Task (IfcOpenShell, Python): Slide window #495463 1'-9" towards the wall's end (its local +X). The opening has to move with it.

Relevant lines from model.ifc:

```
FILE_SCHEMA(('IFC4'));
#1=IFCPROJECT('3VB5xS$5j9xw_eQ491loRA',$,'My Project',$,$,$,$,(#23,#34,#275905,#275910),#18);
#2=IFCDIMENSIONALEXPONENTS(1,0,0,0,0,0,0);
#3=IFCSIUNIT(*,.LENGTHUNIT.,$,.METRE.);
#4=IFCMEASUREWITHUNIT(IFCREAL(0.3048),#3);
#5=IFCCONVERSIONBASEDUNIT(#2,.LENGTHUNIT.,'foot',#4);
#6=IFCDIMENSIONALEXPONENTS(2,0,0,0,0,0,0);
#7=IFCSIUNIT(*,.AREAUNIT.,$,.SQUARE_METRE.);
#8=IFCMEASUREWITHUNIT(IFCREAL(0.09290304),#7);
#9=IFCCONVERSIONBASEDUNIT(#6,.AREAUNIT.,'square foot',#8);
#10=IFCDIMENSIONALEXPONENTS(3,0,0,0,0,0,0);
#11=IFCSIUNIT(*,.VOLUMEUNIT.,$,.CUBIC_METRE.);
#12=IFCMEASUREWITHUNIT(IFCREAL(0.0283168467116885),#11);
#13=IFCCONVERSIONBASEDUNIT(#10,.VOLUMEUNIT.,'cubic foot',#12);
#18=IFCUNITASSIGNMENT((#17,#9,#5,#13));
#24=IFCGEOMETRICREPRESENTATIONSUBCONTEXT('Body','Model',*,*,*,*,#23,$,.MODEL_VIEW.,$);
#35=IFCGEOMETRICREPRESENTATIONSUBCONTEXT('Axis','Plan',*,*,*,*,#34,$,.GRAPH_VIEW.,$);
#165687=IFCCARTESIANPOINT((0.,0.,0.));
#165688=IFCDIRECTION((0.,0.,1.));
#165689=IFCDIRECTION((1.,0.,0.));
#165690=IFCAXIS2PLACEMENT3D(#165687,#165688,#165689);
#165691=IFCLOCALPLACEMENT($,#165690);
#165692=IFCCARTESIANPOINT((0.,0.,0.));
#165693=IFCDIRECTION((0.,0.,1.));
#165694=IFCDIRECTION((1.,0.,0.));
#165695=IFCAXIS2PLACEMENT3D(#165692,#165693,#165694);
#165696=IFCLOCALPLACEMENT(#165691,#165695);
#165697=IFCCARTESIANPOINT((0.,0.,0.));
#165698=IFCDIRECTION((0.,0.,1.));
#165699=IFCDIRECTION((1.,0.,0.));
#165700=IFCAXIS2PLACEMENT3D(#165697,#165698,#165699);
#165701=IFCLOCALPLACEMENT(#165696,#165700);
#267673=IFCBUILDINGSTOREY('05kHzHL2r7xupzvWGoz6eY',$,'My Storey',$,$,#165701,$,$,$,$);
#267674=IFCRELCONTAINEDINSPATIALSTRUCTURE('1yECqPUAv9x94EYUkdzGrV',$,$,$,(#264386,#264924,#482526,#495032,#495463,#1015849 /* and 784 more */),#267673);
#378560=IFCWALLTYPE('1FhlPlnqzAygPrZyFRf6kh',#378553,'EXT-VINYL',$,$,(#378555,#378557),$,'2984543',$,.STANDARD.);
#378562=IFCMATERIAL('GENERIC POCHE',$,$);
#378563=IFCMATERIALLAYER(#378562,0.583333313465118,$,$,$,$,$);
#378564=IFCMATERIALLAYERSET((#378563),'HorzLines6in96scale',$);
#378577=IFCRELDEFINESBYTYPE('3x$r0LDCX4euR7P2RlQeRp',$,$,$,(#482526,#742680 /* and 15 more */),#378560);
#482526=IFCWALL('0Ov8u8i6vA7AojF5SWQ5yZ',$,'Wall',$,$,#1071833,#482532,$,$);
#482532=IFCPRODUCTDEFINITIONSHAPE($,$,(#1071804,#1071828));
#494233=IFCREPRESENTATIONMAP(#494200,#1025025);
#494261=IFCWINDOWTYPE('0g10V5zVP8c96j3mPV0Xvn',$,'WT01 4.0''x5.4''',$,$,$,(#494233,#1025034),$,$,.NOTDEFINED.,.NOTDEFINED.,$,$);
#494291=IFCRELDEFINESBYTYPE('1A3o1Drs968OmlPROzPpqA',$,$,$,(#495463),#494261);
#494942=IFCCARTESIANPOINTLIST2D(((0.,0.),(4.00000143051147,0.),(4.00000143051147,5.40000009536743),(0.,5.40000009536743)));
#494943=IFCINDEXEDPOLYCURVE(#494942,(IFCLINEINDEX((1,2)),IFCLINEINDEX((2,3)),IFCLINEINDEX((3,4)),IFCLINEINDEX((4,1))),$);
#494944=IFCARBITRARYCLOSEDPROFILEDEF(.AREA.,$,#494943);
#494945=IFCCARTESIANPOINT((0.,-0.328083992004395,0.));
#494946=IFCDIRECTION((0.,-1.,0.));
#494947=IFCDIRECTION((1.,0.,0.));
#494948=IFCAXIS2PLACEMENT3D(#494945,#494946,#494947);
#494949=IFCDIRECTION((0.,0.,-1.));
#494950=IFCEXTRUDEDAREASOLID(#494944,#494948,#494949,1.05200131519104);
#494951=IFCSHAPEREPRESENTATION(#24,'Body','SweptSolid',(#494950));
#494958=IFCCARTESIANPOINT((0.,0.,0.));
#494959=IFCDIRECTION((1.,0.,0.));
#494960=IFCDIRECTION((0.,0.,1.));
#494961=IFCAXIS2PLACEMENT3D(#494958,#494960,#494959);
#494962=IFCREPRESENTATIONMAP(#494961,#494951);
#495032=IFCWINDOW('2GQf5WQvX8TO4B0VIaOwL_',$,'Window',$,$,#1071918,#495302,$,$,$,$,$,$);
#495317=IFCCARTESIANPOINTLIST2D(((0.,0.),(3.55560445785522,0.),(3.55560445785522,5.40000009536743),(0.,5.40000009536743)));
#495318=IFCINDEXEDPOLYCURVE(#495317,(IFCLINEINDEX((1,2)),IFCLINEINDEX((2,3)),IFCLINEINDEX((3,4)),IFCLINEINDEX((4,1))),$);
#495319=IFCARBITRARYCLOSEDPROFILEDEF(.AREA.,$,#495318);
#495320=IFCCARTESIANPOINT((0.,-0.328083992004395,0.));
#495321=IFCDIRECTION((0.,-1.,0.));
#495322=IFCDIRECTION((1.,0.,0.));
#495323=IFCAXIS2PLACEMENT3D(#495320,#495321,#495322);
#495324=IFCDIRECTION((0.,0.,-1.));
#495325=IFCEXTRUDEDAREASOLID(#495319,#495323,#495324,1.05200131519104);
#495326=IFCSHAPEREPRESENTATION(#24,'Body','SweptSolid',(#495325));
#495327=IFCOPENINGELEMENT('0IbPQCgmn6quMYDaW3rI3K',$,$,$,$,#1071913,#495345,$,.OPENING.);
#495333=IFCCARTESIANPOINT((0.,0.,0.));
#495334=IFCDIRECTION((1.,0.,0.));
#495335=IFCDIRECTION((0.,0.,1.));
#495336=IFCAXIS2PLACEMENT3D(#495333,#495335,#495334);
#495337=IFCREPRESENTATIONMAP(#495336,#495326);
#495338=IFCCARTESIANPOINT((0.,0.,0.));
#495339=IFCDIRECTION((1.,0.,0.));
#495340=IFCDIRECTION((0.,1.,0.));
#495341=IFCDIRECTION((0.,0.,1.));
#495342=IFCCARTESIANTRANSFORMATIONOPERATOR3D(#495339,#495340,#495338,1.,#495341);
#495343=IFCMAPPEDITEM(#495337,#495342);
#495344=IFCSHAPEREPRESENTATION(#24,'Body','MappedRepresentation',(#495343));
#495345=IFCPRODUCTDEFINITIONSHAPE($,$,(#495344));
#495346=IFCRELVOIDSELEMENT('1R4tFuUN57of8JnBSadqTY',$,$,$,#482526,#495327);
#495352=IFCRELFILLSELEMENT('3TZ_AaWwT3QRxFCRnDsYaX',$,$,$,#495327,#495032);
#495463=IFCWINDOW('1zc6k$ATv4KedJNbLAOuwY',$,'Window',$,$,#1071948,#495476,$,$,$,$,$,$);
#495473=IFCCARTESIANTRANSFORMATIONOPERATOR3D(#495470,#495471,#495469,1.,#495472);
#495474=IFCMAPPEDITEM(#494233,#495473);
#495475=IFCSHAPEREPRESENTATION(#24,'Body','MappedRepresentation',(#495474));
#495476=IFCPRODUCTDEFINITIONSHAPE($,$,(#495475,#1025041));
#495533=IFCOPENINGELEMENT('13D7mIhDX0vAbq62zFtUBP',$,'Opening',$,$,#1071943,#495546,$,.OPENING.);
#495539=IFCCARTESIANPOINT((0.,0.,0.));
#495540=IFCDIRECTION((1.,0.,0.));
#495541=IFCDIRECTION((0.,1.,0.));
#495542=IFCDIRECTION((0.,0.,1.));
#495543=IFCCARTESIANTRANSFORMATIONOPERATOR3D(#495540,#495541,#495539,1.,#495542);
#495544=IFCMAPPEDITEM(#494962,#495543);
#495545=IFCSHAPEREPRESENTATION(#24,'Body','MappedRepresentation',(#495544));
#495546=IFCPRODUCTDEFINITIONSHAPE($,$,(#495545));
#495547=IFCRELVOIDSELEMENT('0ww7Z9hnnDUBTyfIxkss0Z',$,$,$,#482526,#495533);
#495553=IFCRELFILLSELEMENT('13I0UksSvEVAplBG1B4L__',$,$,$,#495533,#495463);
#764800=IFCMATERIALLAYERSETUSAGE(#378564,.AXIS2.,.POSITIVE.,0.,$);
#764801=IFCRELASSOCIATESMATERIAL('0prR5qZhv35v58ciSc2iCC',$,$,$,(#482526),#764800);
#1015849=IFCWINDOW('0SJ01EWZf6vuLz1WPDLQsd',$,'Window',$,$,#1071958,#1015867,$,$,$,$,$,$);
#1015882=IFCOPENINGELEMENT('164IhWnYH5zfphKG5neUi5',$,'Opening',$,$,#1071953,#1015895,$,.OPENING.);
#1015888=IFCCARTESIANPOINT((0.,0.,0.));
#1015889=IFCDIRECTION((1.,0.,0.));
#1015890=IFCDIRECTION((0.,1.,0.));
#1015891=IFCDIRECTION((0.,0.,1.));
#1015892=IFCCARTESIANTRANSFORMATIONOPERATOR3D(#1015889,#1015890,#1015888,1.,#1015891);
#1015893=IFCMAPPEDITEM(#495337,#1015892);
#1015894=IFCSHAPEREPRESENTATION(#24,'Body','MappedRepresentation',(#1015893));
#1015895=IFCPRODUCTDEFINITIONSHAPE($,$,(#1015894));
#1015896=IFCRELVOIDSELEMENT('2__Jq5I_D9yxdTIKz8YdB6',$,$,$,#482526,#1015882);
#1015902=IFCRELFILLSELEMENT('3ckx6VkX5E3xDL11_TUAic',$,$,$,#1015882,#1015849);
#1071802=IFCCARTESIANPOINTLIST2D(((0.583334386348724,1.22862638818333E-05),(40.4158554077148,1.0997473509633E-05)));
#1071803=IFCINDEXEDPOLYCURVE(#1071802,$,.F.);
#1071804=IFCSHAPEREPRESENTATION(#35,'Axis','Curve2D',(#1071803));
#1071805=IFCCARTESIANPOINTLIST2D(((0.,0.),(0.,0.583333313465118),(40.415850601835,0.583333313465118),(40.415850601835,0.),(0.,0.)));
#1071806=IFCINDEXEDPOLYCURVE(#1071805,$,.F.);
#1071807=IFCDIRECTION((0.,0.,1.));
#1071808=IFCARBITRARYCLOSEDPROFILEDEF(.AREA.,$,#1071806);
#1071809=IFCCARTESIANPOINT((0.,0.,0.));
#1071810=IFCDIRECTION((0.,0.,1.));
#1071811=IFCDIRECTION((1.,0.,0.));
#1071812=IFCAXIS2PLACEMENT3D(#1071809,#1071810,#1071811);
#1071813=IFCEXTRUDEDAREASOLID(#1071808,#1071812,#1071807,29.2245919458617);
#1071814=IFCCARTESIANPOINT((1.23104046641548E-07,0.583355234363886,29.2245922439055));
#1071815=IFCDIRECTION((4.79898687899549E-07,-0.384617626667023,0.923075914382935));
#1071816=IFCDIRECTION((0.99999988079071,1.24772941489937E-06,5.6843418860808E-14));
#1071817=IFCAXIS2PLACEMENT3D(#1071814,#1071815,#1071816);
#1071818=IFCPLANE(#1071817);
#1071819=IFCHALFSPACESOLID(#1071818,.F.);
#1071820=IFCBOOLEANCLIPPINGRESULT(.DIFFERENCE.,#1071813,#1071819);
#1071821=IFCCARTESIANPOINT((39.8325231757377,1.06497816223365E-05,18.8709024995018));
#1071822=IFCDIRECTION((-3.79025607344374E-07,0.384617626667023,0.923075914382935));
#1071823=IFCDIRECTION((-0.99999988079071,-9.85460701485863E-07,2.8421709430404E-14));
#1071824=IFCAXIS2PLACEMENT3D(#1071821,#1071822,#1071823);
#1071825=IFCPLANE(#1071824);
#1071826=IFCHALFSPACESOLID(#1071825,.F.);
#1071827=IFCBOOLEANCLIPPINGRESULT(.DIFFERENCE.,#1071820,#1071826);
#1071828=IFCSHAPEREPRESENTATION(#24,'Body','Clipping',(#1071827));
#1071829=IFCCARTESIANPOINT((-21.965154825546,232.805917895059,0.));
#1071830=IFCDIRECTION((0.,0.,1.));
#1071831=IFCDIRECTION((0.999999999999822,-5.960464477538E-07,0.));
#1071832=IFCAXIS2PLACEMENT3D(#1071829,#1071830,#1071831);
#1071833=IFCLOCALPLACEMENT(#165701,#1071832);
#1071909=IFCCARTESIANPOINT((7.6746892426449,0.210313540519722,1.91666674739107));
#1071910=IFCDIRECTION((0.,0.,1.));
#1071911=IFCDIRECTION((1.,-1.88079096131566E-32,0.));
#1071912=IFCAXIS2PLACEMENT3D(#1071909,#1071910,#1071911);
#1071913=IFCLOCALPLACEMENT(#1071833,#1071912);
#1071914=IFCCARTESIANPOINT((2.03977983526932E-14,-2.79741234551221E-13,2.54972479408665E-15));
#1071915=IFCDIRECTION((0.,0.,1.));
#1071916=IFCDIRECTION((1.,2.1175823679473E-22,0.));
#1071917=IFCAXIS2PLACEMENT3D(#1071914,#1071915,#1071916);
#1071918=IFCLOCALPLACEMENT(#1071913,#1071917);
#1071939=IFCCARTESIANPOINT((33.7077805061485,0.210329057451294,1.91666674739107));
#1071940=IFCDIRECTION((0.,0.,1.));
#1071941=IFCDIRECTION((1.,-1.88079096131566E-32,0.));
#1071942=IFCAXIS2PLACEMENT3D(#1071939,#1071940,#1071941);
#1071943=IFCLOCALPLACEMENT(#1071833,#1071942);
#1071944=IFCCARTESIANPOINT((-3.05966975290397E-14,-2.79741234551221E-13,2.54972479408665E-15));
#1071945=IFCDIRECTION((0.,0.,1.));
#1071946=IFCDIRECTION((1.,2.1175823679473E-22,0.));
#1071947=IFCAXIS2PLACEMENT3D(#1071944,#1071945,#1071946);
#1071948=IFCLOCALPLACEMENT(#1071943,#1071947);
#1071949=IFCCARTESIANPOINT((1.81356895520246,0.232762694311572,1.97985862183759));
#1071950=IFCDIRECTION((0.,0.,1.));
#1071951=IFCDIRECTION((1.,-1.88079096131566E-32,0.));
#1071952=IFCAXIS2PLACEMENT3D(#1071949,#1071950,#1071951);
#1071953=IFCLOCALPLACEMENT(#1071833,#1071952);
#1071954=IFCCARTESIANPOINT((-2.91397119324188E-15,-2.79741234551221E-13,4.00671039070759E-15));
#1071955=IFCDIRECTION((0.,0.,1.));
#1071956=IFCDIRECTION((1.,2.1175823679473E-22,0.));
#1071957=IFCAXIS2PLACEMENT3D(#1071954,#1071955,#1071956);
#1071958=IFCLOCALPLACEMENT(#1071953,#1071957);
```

```python
import ifcopenshell
import ifcopenshell.api.geometry
import ifcopenshell.util.placement
import ifcopenshell.util.unit

model = ifcopenshell.open("model.ifc")
unit_scale = ifcopenshell.util.unit.calculate_unit_scale(model)

window = model.by_guid("1zc6k$ATv4KedJNbLAOuwY")
opening = window.FillsVoids[0].RelatingOpeningElement
wall = opening.VoidsElements[0].RelatingBuildingElement

wall_matrix = ifcopenshell.util.placement.get_local_placement(wall.ObjectPlacement)
shift = wall_matrix[:3, 0] * 21 * 0.0254 / unit_scale
before = ifcopenshell.util.placement.get_local_placement(window.ObjectPlacement)[:3, 3].copy()

# The window is placed relative to its opening, so it follows when the opening moves.
matrix = ifcopenshell.util.placement.get_local_placement(opening.ObjectPlacement)
matrix[:3, 3] += shift
ifcopenshell.api.geometry.edit_object_placement(
    model, product=opening, matrix=matrix, is_si=False, should_transform_children=True
)

after = ifcopenshell.util.placement.get_local_placement(window.ObjectPlacement)[:3, 3]
print("window moved by", (after - before).round(3) + 0.0)

model.write("model_v2.ifc")
```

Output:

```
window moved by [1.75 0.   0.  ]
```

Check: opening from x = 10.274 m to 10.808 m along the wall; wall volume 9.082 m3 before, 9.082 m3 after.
